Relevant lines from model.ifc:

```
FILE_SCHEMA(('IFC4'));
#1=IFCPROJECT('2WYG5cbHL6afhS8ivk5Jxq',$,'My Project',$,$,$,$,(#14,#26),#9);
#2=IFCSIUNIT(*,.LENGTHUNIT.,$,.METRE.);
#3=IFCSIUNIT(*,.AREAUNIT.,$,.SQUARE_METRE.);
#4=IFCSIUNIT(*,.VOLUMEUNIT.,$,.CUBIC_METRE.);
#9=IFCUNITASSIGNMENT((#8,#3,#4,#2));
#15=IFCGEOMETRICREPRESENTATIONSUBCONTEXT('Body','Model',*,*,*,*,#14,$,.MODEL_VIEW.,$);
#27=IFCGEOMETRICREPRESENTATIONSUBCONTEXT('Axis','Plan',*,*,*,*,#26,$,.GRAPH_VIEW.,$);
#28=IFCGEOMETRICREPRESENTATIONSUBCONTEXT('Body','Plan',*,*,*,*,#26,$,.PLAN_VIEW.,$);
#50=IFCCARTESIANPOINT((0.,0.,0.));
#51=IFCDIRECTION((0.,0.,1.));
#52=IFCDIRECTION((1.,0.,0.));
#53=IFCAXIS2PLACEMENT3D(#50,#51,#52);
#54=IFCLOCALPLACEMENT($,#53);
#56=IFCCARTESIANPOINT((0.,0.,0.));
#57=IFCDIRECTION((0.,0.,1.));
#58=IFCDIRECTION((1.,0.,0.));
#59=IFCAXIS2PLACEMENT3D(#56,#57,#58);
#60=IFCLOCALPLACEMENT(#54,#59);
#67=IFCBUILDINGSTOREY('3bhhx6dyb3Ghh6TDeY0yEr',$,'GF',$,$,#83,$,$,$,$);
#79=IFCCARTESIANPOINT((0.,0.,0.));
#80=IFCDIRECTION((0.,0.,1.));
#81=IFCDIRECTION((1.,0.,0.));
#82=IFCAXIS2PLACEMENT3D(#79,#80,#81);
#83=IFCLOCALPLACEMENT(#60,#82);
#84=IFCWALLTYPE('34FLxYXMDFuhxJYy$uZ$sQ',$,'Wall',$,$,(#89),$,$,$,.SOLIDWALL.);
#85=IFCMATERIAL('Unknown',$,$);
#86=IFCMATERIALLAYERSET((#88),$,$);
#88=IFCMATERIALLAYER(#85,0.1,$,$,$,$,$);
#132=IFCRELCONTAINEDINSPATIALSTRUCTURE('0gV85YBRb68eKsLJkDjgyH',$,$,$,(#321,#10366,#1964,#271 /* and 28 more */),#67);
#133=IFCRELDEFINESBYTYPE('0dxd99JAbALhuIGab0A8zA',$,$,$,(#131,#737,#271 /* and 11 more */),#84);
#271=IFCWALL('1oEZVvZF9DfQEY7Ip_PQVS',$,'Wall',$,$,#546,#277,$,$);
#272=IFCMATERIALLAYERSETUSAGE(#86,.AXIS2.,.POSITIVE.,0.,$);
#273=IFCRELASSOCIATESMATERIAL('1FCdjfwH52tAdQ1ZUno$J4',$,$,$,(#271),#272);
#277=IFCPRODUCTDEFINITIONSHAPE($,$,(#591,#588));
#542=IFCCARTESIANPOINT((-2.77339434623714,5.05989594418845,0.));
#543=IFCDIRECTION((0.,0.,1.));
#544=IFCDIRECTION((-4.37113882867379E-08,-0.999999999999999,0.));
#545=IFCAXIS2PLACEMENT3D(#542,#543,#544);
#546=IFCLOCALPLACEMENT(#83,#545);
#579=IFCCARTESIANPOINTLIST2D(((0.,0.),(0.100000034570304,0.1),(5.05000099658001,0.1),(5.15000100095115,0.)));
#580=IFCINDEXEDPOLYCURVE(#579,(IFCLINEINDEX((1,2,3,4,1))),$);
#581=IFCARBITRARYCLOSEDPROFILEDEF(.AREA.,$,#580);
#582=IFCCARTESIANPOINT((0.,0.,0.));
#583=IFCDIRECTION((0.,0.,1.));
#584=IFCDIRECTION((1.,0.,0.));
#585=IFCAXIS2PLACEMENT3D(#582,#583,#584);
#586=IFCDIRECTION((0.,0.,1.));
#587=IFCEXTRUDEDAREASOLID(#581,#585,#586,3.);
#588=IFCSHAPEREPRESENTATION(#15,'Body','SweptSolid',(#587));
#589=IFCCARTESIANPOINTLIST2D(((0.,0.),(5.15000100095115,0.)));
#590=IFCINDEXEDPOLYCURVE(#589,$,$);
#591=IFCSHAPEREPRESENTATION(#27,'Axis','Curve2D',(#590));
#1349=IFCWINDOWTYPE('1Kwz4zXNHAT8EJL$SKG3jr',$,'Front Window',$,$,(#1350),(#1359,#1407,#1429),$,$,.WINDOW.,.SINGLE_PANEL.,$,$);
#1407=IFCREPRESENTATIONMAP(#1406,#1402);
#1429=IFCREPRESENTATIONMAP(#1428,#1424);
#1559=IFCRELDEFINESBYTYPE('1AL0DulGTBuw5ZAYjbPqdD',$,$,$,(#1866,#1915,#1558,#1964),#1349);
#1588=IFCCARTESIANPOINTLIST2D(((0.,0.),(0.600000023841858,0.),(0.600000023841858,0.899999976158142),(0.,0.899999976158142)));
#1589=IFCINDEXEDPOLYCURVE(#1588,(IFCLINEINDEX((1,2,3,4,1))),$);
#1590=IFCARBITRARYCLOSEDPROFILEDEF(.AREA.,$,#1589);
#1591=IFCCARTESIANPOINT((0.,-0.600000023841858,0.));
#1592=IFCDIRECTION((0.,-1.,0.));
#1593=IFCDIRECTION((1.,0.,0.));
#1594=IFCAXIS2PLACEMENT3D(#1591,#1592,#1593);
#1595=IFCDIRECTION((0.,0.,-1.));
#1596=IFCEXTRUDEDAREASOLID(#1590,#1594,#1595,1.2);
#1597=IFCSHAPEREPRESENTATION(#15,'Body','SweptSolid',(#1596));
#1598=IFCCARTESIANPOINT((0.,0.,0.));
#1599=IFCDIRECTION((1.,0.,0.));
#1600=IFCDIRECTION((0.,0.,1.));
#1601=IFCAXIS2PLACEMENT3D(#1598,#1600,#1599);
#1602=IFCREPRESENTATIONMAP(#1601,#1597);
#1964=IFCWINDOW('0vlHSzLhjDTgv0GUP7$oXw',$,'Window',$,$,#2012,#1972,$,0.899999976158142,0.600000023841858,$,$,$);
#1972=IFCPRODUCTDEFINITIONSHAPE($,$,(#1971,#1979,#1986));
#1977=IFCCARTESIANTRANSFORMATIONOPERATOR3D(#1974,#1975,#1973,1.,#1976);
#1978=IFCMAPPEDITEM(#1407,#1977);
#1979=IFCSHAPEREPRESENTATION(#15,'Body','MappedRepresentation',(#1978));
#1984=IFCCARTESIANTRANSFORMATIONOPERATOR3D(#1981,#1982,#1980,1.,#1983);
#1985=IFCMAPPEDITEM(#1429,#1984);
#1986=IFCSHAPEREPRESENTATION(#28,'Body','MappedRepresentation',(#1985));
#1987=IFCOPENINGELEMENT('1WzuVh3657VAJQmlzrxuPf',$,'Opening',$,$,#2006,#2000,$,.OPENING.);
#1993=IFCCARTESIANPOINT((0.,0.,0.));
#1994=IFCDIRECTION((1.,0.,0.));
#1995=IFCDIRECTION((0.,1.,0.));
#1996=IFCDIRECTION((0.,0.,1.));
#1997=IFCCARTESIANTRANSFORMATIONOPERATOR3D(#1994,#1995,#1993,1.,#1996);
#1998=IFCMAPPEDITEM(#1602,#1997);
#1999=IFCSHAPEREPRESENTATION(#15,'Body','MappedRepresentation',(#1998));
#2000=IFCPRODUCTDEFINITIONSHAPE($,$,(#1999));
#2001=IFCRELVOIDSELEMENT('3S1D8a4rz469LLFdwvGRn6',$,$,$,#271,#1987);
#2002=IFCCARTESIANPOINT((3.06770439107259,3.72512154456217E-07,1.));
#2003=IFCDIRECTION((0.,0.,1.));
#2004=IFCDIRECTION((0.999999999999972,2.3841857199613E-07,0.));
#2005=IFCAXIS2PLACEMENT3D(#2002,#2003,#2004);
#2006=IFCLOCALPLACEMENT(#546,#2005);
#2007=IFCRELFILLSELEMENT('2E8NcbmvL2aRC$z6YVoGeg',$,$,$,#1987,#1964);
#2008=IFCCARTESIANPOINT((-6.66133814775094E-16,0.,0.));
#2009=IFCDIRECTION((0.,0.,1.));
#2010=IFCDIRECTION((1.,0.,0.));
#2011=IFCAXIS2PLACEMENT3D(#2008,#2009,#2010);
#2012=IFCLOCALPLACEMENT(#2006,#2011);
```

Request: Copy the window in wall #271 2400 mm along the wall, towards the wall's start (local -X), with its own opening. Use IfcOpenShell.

```python
import ifcopenshell
import ifcopenshell.api.feature
import ifcopenshell.api.geometry
import ifcopenshell.api.root
import ifcopenshell.geom
import ifcopenshell.util.element
import ifcopenshell.util.placement
import ifcopenshell.util.shape
import ifcopenshell.util.unit

model = ifcopenshell.open("model.ifc")
unit_scale = ifcopenshell.util.unit.calculate_unit_scale(model)
settings = ifcopenshell.geom.settings()


def volume(element):
    """Net volume in cubic metres, openings subtracted."""
    shape = ifcopenshell.geom.create_shape(settings, element)
    return ifcopenshell.util.shape.get_volume(shape.geometry)


window = model.by_guid("0vlHSzLhjDTgv0GUP7$oXw")
opening = window.FillsVoids[0].RelatingOpeningElement
wall = opening.VoidsElements[0].RelatingBuildingElement
before = volume(wall)
shift = ifcopenshell.util.placement.get_local_placement(wall.ObjectPlacement)[:3, 0] * -2.4 / unit_scale

# copy_class copies the void relationship, type, container and properties, but no geometry.
new_opening = ifcopenshell.api.root.copy_class(model, product=opening)
new_opening.Representation = ifcopenshell.util.element.copy_deep(
    model, opening.Representation, exclude=["IfcGeometricRepresentationContext", "IfcRepresentationMap"]
)
new_window = ifcopenshell.api.root.copy_class(model, product=window)
new_window.Representation = ifcopenshell.util.element.copy_deep(
    model, window.Representation, exclude=["IfcGeometricRepresentationContext", "IfcRepresentationMap"]
)
ifcopenshell.api.feature.add_filling(model, opening=new_opening, element=new_window)

for old, new in ((opening, new_opening), (window, new_window)):
    matrix = ifcopenshell.util.placement.get_local_placement(old.ObjectPlacement)
    matrix[:3, 3] += shift
    ifcopenshell.api.geometry.edit_object_placement(model, product=new, matrix=matrix, is_si=False)

after = volume(wall)

print(f"wall volume {before:.3f} -> {after:.3f} m3")

model.write("model_edited.ifc")
```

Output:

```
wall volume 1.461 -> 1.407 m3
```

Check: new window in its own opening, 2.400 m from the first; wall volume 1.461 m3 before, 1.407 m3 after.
